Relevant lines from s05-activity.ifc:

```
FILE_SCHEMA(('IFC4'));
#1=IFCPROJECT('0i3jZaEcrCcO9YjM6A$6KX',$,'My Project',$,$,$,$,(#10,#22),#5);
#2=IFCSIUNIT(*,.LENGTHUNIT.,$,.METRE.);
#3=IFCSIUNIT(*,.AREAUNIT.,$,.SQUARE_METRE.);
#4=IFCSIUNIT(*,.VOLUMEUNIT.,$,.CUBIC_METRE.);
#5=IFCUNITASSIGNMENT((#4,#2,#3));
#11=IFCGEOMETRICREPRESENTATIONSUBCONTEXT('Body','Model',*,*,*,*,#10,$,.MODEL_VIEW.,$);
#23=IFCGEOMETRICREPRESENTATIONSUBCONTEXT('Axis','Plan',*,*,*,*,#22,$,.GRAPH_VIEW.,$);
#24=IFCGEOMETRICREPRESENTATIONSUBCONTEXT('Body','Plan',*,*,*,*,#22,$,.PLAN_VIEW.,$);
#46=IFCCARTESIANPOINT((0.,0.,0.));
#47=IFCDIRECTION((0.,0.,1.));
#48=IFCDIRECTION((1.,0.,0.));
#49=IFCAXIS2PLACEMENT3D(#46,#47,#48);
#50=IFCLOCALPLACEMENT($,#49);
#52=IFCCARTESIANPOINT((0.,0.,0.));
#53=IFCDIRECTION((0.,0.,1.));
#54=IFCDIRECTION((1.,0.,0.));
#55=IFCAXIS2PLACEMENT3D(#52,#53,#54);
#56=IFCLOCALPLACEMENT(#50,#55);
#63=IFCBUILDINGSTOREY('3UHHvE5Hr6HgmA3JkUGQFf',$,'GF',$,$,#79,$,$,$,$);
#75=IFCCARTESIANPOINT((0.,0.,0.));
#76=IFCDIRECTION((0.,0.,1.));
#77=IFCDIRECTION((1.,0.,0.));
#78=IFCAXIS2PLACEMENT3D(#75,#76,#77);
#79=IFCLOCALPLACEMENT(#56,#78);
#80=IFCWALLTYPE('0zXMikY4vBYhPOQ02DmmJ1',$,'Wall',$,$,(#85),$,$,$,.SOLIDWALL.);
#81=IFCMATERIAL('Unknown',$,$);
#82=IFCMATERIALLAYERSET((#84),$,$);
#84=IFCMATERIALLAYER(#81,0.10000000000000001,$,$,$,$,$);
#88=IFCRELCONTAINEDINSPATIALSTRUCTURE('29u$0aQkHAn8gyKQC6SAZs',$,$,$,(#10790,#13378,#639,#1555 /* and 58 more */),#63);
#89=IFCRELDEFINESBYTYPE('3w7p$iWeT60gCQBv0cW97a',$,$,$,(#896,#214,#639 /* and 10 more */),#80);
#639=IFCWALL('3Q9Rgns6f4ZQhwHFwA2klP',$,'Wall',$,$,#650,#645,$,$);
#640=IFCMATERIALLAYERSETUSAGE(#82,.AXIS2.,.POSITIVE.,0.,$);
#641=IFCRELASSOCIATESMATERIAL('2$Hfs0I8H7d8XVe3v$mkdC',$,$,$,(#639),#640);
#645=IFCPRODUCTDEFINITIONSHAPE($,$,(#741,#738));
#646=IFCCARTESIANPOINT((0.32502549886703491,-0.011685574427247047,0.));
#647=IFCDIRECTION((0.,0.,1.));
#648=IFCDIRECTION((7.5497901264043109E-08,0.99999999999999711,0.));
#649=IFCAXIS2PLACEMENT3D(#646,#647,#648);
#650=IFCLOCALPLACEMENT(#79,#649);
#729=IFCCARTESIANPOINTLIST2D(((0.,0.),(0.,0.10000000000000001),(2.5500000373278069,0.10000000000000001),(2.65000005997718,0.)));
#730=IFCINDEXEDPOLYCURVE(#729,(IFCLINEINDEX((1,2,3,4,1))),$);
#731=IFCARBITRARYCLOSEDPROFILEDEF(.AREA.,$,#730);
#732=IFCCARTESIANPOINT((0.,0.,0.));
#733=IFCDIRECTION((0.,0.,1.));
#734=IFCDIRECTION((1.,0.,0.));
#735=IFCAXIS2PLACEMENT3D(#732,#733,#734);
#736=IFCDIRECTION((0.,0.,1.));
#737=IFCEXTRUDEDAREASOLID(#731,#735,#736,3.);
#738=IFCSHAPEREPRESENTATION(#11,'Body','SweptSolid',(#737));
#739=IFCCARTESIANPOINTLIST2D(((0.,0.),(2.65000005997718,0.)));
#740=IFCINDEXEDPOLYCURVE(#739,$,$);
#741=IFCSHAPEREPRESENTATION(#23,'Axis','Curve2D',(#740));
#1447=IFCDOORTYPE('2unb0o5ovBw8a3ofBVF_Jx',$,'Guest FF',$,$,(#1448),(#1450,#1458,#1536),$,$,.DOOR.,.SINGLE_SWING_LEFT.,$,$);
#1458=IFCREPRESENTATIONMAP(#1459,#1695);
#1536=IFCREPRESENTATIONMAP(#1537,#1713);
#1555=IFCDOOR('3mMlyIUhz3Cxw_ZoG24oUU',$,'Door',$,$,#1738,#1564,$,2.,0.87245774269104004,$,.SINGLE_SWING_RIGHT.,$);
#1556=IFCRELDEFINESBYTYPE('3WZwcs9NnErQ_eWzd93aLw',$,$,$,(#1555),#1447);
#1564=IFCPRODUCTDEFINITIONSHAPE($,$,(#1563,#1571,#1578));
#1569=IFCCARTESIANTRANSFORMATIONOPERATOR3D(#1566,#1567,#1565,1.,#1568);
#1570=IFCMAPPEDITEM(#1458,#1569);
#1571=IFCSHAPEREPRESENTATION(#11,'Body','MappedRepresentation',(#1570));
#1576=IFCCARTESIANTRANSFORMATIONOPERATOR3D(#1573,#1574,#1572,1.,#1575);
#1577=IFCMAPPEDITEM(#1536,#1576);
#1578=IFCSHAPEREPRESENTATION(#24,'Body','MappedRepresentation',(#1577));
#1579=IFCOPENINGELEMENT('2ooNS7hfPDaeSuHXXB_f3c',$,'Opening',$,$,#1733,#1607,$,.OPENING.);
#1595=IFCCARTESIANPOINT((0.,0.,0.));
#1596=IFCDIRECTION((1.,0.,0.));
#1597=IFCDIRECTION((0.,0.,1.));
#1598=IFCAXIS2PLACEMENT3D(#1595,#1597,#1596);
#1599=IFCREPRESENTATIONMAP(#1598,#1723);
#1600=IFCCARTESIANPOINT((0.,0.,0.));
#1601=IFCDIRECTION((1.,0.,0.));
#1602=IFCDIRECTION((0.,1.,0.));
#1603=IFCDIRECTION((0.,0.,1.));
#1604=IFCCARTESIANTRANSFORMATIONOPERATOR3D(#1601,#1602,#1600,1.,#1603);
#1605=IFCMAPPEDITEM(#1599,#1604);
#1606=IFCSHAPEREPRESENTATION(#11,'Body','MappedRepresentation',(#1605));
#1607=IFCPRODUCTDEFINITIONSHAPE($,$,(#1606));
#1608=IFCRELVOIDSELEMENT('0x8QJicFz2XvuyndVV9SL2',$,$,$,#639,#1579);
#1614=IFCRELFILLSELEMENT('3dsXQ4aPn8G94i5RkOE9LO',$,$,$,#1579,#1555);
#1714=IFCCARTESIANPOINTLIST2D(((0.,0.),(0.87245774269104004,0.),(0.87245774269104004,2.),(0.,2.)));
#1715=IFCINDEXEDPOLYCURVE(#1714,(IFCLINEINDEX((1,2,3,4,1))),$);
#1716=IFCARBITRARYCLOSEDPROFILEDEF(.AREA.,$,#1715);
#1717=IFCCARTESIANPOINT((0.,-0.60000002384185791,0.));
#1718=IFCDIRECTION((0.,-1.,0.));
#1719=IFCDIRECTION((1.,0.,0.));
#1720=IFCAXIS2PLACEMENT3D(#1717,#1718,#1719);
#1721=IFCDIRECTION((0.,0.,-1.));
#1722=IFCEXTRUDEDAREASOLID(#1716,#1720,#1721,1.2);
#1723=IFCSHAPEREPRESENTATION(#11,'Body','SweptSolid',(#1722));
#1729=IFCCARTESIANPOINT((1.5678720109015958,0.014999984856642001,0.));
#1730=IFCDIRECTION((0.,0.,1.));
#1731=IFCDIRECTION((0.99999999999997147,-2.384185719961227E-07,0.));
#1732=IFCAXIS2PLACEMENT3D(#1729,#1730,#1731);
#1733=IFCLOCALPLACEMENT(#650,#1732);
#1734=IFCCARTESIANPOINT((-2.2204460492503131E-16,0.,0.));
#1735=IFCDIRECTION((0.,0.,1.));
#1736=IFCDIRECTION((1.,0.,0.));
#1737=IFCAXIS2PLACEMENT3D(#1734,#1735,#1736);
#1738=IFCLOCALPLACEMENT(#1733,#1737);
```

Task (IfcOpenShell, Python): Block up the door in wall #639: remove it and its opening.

```python
import ifcopenshell
import ifcopenshell.api.feature
import ifcopenshell.api.root
import ifcopenshell.geom
import ifcopenshell.util.shape

model = ifcopenshell.open("s05-activity.ifc")
settings = ifcopenshell.geom.settings()


def volume(element):
    """Net volume in cubic metres, openings subtracted."""
    shape = ifcopenshell.geom.create_shape(settings, element)
    return ifcopenshell.util.shape.get_volume(shape.geometry)


door = model.by_id(1555)
opening = door.FillsVoids[0].RelatingOpeningElement
wall = opening.VoidsElements[0].RelatingBuildingElement
before = volume(wall)

ifcopenshell.api.root.remove_product(model, product=door)
ifcopenshell.api.feature.remove_feature(model, feature=opening)

after = volume(wall)

print(f"wall volume {before:.3f} -> {after:.3f} m3")

model.write("s05-activity_updated.ifc")
```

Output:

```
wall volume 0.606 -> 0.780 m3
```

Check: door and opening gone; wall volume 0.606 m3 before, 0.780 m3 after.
